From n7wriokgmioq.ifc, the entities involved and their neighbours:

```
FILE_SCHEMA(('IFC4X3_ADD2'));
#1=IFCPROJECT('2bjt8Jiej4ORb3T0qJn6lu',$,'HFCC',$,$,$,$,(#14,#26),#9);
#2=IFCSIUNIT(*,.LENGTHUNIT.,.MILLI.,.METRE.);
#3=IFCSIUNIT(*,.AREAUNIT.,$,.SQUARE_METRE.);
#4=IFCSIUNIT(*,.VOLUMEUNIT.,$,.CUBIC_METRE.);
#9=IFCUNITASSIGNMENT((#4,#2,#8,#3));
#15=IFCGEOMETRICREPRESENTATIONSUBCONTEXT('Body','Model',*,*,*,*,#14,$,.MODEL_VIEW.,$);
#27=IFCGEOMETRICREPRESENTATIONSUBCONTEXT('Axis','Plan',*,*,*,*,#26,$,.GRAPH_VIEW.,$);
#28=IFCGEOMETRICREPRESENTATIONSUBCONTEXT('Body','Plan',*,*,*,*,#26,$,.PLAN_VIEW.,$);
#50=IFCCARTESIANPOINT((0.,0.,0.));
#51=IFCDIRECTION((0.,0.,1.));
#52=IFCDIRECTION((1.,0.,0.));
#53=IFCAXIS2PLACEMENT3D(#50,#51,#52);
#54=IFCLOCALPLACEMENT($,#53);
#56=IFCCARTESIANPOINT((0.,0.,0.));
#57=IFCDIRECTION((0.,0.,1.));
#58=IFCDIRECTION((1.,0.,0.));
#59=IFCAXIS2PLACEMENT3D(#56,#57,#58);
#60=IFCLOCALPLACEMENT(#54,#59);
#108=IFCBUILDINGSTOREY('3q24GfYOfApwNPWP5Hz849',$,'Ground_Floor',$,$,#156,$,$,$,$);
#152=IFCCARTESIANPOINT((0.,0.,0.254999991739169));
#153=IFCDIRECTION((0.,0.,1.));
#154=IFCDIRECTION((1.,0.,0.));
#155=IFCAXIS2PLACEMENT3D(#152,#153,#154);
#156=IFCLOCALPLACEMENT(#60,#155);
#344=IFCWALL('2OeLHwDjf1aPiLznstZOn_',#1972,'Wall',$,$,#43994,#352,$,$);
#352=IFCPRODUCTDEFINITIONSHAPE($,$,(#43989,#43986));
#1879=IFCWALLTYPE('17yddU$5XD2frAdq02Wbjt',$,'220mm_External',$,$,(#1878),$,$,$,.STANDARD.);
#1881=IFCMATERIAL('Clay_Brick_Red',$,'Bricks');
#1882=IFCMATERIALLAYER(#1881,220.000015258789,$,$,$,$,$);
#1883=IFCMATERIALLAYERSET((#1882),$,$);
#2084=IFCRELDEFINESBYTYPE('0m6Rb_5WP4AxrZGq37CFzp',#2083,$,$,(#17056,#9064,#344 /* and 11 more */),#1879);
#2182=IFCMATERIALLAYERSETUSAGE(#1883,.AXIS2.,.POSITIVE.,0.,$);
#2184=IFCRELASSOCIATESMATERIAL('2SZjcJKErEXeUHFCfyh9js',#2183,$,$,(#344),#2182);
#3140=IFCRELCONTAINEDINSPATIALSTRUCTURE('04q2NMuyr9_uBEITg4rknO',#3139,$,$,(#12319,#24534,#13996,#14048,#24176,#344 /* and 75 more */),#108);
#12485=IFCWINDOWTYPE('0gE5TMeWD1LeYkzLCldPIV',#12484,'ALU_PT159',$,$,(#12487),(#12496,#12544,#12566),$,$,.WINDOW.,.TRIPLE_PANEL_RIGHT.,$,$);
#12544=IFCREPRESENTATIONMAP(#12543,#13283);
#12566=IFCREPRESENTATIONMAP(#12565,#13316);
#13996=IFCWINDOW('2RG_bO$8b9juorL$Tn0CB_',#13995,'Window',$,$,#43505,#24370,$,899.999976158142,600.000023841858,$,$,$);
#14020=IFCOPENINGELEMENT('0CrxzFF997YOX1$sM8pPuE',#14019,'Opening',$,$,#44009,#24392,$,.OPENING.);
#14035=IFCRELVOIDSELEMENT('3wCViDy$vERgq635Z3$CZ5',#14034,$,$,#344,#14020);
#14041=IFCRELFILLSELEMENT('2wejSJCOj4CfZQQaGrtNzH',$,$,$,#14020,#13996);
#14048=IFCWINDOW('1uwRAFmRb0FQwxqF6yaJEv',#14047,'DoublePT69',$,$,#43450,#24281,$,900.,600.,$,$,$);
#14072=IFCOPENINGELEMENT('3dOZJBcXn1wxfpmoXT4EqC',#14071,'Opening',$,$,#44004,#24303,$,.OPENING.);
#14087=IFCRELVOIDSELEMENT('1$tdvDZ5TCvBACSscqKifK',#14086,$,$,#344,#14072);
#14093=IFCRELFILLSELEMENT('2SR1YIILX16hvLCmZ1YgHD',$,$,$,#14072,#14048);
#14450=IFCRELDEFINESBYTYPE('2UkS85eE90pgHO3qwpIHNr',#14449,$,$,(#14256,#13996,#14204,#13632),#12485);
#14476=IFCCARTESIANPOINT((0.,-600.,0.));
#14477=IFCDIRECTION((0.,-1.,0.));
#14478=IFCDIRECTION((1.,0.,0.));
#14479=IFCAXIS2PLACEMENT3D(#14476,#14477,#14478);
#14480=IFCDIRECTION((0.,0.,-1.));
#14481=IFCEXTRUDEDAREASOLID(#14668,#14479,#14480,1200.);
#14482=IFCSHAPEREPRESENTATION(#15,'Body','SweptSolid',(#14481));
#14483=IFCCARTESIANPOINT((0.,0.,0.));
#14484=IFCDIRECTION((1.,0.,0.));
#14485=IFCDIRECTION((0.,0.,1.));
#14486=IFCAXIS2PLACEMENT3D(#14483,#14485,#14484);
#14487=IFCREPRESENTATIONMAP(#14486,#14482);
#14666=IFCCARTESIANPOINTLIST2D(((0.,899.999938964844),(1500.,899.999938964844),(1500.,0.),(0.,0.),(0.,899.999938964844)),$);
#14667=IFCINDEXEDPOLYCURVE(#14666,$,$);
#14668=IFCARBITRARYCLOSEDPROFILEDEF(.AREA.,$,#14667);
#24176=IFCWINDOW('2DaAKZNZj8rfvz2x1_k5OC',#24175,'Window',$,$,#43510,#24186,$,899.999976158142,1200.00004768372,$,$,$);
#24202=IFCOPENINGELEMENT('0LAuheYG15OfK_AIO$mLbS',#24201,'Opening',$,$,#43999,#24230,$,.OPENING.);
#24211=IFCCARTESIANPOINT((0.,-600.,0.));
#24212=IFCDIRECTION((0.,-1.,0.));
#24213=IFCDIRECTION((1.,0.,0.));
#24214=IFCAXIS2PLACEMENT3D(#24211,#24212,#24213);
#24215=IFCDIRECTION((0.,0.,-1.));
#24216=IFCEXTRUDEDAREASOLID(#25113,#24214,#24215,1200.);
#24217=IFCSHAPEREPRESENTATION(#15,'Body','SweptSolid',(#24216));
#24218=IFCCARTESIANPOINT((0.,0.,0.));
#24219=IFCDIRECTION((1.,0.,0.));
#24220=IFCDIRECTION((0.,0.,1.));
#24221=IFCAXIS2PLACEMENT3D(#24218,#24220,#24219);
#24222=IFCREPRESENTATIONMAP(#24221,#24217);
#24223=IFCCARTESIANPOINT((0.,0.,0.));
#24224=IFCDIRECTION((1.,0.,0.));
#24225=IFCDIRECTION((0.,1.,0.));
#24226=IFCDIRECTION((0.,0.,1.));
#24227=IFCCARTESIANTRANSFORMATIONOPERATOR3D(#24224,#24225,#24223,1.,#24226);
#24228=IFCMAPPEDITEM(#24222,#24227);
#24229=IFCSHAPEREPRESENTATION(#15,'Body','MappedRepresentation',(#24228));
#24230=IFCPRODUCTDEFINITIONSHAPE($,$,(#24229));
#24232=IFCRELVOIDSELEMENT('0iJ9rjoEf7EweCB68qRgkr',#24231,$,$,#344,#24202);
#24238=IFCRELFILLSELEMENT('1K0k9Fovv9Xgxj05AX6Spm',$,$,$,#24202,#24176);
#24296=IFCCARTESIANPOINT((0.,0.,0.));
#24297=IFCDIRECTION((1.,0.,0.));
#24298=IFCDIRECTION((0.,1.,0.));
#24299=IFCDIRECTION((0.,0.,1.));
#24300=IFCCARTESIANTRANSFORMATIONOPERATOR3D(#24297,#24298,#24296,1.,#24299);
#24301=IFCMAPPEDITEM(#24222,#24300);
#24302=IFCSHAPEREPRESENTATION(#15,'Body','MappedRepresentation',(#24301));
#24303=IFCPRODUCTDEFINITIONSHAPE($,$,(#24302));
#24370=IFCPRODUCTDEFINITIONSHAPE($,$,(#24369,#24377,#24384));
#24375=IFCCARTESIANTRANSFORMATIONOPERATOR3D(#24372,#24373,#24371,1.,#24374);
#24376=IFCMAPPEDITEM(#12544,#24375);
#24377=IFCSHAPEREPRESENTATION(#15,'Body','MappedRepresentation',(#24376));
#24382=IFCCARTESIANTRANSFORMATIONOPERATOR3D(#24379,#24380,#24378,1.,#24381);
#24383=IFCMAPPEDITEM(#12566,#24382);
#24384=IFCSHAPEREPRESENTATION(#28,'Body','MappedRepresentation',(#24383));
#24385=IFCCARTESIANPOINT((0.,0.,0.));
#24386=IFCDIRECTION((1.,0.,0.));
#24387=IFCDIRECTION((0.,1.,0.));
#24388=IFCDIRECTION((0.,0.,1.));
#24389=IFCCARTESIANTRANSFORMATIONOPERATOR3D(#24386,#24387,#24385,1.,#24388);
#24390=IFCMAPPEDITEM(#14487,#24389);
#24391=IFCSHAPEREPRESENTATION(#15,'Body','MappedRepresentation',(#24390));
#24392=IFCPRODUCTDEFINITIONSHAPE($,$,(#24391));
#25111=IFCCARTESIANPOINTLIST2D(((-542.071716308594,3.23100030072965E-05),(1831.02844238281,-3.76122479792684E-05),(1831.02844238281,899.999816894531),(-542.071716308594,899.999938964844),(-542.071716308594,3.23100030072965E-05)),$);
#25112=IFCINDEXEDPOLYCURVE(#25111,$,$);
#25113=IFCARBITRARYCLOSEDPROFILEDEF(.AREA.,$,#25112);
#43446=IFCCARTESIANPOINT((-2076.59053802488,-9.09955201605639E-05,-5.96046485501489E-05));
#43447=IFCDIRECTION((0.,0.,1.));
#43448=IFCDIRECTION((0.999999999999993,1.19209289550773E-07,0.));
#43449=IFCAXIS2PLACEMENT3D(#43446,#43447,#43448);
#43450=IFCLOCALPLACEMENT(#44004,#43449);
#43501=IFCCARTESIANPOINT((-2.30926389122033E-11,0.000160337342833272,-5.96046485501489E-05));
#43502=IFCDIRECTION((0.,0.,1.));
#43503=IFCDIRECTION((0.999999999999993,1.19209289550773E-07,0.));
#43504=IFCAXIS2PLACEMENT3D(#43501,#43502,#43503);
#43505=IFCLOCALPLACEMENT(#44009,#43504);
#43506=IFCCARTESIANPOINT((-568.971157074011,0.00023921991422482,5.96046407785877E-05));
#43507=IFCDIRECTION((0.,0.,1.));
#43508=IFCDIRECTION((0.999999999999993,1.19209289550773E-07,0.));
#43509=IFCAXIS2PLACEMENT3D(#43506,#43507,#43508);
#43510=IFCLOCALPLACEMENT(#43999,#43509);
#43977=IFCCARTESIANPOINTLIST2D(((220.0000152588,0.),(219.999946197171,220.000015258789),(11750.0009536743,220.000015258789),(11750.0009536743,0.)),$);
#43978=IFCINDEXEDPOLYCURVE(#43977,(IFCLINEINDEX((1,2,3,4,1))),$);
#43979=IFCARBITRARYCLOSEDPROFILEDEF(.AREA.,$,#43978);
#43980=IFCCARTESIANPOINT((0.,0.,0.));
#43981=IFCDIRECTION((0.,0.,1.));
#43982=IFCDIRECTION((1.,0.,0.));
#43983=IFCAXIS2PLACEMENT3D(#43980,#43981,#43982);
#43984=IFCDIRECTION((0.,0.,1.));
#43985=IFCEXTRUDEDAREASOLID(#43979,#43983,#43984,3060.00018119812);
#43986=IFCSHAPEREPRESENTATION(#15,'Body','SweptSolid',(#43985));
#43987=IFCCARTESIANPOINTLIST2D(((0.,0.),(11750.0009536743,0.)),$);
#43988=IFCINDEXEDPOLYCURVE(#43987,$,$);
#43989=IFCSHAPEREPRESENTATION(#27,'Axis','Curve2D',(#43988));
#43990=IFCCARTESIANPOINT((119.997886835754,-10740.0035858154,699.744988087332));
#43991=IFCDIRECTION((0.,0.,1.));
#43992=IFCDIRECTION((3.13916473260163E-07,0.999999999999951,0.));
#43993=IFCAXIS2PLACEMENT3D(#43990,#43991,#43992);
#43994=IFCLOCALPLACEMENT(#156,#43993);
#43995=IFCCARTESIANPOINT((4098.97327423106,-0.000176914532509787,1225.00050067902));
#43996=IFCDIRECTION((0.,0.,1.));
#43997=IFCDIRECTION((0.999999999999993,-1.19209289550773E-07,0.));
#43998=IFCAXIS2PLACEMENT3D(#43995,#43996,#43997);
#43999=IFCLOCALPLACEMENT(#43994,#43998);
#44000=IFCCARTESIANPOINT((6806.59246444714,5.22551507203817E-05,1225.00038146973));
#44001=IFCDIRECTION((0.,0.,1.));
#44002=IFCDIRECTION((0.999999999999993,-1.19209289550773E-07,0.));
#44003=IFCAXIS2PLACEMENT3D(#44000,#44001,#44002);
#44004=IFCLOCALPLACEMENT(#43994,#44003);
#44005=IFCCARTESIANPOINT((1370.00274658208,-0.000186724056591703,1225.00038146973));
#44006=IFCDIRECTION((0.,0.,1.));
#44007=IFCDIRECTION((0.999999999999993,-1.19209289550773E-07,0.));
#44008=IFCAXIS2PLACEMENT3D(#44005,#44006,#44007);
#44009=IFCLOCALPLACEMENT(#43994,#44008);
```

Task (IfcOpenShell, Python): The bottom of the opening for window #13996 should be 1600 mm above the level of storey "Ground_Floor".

```python
import numpy as np
import ifcopenshell
import ifcopenshell.api.geometry
import ifcopenshell.geom
import ifcopenshell.util.element
import ifcopenshell.util.placement
import ifcopenshell.util.shape
import ifcopenshell.util.unit

model = ifcopenshell.open("n7wriokgmioq.ifc")
unit_scale = ifcopenshell.util.unit.calculate_unit_scale(model)

window = model.by_guid("2RG_bO$8b9juorL$Tn0CB_")
opening = window.FillsVoids[0].RelatingOpeningElement
storey = ifcopenshell.util.element.get_container(window, ifc_class="IfcBuildingStorey")
level = ifcopenshell.util.placement.get_local_placement(storey.ObjectPlacement)[2, 3]

# The opening's origin need not be at the sill, so measure its lowest point.
shape = ifcopenshell.geom.create_shape(ifcopenshell.geom.settings(), opening)
bottom = ifcopenshell.util.shape.get_shape_bottom_elevation(shape, shape.geometry) / unit_scale
dz = level + 1.6 / unit_scale - bottom

shift = np.array([0.0, 0.0, dz])
# The window is placed relative to its opening, so it follows when the opening moves.
matrix = ifcopenshell.util.placement.get_local_placement(opening.ObjectPlacement)
matrix[:3, 3] += shift
ifcopenshell.api.geometry.edit_object_placement(
    model, product=opening, matrix=matrix, is_si=False, should_transform_children=True
)

print(f"moved by {dz * unit_scale:+.3f} m")

model.write("n7wriokgmioq_rev.ifc")
```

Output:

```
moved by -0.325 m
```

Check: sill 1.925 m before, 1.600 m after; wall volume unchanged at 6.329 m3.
